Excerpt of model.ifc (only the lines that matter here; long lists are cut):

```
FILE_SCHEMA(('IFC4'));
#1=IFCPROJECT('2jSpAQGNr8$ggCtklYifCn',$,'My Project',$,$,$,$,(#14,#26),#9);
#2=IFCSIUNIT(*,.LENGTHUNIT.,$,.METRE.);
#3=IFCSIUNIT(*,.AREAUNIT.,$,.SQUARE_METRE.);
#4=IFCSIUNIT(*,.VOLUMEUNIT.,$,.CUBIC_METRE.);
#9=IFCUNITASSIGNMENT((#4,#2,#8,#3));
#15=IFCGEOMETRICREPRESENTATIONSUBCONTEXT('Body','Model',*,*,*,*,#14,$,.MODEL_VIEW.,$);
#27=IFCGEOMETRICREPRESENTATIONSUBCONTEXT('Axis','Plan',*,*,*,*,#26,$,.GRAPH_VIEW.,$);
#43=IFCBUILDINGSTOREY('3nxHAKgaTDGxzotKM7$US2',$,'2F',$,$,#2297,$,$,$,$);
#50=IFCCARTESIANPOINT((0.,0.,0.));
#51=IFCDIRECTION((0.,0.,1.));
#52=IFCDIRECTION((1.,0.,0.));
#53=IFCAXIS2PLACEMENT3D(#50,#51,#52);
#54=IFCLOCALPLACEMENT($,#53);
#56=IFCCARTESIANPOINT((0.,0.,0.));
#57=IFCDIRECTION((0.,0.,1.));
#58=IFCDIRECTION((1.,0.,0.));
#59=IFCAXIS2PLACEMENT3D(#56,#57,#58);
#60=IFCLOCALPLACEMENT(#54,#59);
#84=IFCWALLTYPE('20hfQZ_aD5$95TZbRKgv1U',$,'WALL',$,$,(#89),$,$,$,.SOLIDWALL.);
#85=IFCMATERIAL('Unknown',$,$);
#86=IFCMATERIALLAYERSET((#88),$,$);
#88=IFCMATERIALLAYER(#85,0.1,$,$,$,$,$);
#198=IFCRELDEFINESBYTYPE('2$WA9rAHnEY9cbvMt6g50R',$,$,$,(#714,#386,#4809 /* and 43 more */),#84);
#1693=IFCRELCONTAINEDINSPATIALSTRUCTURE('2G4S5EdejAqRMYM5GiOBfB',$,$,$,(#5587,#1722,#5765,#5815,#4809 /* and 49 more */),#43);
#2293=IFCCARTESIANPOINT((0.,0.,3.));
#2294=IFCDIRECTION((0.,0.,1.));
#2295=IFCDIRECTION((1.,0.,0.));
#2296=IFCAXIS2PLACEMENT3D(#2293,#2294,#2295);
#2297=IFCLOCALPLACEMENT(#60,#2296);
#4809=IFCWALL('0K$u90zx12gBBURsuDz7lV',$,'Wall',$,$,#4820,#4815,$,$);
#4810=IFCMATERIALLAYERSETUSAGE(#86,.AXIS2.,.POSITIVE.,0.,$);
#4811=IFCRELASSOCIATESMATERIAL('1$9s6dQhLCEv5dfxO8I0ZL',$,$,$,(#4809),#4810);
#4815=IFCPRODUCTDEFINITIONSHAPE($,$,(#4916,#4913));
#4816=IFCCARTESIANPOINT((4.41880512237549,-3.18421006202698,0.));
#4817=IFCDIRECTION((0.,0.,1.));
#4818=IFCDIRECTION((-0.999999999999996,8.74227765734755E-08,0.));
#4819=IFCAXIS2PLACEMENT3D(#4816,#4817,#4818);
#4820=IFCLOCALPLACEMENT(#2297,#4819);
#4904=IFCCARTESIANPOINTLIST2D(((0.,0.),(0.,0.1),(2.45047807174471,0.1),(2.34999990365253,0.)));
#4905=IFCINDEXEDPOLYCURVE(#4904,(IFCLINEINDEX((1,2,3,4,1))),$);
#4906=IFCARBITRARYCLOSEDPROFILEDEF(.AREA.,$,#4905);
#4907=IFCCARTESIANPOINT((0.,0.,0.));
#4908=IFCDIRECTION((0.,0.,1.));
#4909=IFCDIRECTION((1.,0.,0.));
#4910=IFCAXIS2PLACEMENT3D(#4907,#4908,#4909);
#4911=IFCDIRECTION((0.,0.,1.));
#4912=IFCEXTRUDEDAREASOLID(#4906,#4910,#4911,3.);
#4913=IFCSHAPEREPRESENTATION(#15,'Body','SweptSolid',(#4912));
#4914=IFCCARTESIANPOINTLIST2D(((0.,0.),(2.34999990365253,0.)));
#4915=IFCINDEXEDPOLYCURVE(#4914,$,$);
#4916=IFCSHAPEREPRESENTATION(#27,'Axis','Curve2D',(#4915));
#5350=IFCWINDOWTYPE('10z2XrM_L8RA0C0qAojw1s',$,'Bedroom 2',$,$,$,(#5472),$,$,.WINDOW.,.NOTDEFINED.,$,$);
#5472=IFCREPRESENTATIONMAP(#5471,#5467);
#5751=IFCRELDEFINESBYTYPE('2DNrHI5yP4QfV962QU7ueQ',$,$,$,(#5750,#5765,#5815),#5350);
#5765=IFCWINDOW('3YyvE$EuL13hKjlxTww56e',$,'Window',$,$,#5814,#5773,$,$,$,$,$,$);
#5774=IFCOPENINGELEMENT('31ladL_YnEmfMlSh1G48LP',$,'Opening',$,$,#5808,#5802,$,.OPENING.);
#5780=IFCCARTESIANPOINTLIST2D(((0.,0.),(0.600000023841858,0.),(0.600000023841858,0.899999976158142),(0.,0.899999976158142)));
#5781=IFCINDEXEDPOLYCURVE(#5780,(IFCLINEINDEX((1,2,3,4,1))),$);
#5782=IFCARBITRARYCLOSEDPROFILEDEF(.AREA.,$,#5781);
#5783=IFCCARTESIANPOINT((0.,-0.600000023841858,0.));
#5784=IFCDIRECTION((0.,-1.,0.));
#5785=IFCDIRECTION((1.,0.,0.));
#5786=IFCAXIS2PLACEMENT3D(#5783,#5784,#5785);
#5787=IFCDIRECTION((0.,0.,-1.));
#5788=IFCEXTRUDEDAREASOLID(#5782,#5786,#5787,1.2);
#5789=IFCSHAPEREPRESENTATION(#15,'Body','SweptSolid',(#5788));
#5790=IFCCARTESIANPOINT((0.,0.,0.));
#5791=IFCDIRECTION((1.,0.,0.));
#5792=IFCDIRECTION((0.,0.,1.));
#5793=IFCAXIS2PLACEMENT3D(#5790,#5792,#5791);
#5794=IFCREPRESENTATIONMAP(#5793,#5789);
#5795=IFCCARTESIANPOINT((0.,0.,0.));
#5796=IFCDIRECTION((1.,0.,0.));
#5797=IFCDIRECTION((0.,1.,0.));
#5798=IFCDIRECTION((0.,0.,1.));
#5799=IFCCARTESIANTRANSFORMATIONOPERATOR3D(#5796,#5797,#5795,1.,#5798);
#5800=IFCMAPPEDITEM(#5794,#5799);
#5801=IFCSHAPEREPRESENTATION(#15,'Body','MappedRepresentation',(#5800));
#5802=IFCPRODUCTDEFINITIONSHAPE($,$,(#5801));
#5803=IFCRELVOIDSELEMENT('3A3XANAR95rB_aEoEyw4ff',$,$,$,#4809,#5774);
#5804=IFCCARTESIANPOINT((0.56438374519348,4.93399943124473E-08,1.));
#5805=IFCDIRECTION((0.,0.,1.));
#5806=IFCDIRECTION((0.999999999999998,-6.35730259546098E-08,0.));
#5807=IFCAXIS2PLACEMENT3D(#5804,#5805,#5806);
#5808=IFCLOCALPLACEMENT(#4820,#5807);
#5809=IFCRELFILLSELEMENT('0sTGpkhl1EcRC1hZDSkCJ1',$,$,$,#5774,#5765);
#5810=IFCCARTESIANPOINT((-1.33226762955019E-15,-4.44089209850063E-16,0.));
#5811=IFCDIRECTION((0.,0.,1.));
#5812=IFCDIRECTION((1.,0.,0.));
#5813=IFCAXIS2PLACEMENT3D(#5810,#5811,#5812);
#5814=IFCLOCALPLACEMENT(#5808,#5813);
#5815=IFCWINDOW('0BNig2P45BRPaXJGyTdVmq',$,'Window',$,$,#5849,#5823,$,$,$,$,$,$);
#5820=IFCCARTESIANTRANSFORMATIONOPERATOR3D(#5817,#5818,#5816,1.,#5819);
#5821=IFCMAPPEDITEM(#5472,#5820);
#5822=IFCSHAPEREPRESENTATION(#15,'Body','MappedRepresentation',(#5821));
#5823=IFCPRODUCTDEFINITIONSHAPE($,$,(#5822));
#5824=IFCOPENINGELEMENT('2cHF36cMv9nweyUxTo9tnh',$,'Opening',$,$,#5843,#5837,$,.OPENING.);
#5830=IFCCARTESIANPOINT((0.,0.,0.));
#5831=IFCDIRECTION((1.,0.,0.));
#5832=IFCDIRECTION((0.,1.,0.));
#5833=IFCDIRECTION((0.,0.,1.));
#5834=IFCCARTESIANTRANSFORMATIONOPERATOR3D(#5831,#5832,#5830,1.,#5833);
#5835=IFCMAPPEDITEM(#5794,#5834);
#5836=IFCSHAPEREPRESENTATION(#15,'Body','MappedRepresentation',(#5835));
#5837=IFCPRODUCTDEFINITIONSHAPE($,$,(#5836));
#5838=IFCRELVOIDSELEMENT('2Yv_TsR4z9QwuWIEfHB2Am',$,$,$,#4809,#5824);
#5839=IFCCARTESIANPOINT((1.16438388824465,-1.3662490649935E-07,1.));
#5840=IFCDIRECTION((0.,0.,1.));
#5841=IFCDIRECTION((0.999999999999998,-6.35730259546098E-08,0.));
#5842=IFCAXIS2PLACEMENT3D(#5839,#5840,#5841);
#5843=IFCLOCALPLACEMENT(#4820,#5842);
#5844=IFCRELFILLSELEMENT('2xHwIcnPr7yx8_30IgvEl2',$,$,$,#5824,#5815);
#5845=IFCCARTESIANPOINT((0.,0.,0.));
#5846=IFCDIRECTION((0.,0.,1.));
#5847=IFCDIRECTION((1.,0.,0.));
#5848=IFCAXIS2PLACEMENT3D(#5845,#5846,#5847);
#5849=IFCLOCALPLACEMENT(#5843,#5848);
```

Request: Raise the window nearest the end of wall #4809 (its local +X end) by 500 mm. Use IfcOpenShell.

```python
import numpy as np
import ifcopenshell
import ifcopenshell.api.geometry
import ifcopenshell.util.placement
import ifcopenshell.util.unit

model = ifcopenshell.open("model.ifc")
unit_scale = ifcopenshell.util.unit.calculate_unit_scale(model)

window = model.by_id(5815)
opening = window.FillsVoids[0].RelatingOpeningElement
dz = 0.5 / unit_scale

shift = np.array([0.0, 0.0, dz])
# The window is placed relative to its opening, so it follows when the opening moves.
matrix = ifcopenshell.util.placement.get_local_placement(opening.ObjectPlacement)
matrix[:3, 3] += shift
ifcopenshell.api.geometry.edit_object_placement(
    model, product=opening, matrix=matrix, is_si=False, should_transform_children=True
)

print(f"moved by {dz * unit_scale:+.3f} m")

model.write("model_rev.ifc")
```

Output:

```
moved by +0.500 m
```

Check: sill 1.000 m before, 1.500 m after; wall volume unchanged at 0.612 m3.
